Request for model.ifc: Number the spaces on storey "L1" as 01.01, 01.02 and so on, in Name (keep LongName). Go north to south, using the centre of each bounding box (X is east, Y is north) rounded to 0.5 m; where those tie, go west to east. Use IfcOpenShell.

First a look at what the model holds.

```python
import ifcopenshell
import ifcopenshell.util.element
import ifcopenshell.util.placement

model = ifcopenshell.open("model.ifc")
print(model.schema)
storey = next(s for s in model.by_type("IfcBuildingStorey") if s.Name == "L1")
spaces = [e for e in ifcopenshell.util.element.get_decomposition(storey) if e.is_a("IfcSpace")]
for e in sorted(spaces, key=lambda e: e.id()):
    origin = ifcopenshell.util.placement.get_local_placement(e.ObjectPlacement)[:3, 3]
    print(e.id(), e.Name, e.LongName, origin.round(2) + 0.0, sep=" | ")
```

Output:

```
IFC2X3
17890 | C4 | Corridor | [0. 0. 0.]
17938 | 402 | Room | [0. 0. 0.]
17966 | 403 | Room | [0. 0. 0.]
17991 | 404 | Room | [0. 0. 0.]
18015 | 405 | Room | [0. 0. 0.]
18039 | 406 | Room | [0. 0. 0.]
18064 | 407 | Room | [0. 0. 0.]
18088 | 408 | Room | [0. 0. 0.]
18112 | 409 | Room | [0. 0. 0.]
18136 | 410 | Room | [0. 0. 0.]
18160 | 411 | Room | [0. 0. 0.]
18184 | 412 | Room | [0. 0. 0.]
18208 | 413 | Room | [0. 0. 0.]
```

```python
import ifcopenshell
import ifcopenshell.geom
import ifcopenshell.util.element
import ifcopenshell.util.shape

model = ifcopenshell.open("model.ifc")
settings = ifcopenshell.geom.settings()
settings.set("use-world-coords", True)


def centre(element):
    shape = ifcopenshell.geom.create_shape(settings, element)
    return ifcopenshell.util.shape.get_bbox_centroid(shape.geometry)


storey = next(s for s in model.by_type("IfcBuildingStorey") if s.Name == "L1")
spaces = [e for e in ifcopenshell.util.element.get_decomposition(storey) if e.is_a("IfcSpace")]

# Insertion points can sit at a corner or the storey origin, so sort by the geometry (in metres).
centres = {e: centre(e) for e in spaces}
spaces.sort(key=lambda e: (-round(centres[e][1] / 0.5), centres[e][0]))

for i, e in enumerate(spaces, start=1):
    number = f"01.{i:02d}"
    e.Name = number
    print(e.id(), number)

model.write("model_updated.ifc")
```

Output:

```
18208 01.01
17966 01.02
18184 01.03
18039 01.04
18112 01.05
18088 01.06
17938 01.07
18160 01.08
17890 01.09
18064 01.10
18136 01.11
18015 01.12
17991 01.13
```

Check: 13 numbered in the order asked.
